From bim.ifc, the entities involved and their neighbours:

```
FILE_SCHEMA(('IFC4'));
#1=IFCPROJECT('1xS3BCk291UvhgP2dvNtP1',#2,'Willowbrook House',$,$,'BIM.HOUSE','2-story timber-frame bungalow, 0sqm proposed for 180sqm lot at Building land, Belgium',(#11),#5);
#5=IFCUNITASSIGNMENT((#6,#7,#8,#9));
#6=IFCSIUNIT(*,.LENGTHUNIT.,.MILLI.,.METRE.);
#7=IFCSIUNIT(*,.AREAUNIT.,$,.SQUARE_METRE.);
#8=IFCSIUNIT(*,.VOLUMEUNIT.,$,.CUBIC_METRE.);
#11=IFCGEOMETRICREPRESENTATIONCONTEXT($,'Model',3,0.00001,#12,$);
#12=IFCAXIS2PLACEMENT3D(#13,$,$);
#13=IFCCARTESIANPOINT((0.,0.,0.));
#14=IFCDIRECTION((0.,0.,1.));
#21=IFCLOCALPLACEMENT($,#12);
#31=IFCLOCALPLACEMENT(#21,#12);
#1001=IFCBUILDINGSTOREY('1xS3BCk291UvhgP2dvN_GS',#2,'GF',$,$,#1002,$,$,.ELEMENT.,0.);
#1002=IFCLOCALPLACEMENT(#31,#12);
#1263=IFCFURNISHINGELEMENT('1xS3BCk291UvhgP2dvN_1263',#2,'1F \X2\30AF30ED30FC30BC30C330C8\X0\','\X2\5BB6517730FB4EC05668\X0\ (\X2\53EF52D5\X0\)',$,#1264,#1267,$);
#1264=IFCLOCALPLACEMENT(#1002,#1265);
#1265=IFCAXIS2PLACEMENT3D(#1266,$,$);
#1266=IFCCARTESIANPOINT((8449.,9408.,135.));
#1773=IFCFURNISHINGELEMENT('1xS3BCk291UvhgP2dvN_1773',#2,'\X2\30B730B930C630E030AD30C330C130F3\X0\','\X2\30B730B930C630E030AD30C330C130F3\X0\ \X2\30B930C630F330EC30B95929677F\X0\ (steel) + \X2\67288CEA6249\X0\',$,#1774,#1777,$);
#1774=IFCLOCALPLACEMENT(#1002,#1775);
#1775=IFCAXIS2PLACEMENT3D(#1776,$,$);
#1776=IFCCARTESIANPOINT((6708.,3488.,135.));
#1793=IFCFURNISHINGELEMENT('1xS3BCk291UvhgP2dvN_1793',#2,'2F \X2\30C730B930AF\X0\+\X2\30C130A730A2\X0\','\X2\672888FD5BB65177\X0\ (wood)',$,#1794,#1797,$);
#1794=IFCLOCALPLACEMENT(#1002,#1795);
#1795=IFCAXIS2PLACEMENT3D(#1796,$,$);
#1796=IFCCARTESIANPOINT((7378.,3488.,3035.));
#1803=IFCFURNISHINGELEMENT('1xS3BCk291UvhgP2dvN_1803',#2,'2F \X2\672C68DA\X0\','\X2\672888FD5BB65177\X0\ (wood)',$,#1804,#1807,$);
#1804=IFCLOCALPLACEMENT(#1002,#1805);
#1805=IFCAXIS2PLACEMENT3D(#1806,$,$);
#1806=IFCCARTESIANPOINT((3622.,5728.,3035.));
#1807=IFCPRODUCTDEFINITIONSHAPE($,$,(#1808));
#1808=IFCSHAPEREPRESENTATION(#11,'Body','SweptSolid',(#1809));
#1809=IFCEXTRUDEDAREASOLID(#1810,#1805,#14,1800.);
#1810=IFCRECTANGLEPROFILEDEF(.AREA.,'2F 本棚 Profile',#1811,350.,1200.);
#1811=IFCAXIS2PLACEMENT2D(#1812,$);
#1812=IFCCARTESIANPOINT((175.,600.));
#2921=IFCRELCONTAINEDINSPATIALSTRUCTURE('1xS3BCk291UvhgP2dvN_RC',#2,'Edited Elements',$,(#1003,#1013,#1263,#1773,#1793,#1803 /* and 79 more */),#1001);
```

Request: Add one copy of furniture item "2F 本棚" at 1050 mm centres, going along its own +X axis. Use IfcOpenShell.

```python
import ifcopenshell
import ifcopenshell.api.geometry
import ifcopenshell.api.root
import ifcopenshell.util.element
import ifcopenshell.util.placement

model = ifcopenshell.open("bim.ifc")


def reuse_history(source, copy):
    """copy_class also copies each property set's owner history, people and application; keep the originals."""
    for rel in copy.IsDefinedBy:
        if rel.is_a("IfcRelDefinesByProperties") and (history := rel.RelatingPropertyDefinition.OwnerHistory):
            rel.RelatingPropertyDefinition.OwnerHistory = source.OwnerHistory
            ifcopenshell.util.element.remove_deep2(model, history)


source = model.by_id(1803)
base = ifcopenshell.util.placement.get_local_placement(source.ObjectPlacement)
step = base[:3, 0] * 1050.0

for i in range(1, 2):
    copy = ifcopenshell.api.root.copy_class(model, product=source)
    copy.Representation = ifcopenshell.util.element.copy_deep(
        model, source.Representation, exclude=["IfcGeometricRepresentationContext", "IfcRepresentationMap"]
    )
    reuse_history(source, copy)
    matrix = base.copy()
    matrix[:3, 3] += i * step
    print("added at", matrix[:3, 3].round(3) + 0.0)
    ifcopenshell.api.geometry.edit_object_placement(model, product=copy, matrix=matrix, is_si=False)

model.write("bim-out.ifc")
```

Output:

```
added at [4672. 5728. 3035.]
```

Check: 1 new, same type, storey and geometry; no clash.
